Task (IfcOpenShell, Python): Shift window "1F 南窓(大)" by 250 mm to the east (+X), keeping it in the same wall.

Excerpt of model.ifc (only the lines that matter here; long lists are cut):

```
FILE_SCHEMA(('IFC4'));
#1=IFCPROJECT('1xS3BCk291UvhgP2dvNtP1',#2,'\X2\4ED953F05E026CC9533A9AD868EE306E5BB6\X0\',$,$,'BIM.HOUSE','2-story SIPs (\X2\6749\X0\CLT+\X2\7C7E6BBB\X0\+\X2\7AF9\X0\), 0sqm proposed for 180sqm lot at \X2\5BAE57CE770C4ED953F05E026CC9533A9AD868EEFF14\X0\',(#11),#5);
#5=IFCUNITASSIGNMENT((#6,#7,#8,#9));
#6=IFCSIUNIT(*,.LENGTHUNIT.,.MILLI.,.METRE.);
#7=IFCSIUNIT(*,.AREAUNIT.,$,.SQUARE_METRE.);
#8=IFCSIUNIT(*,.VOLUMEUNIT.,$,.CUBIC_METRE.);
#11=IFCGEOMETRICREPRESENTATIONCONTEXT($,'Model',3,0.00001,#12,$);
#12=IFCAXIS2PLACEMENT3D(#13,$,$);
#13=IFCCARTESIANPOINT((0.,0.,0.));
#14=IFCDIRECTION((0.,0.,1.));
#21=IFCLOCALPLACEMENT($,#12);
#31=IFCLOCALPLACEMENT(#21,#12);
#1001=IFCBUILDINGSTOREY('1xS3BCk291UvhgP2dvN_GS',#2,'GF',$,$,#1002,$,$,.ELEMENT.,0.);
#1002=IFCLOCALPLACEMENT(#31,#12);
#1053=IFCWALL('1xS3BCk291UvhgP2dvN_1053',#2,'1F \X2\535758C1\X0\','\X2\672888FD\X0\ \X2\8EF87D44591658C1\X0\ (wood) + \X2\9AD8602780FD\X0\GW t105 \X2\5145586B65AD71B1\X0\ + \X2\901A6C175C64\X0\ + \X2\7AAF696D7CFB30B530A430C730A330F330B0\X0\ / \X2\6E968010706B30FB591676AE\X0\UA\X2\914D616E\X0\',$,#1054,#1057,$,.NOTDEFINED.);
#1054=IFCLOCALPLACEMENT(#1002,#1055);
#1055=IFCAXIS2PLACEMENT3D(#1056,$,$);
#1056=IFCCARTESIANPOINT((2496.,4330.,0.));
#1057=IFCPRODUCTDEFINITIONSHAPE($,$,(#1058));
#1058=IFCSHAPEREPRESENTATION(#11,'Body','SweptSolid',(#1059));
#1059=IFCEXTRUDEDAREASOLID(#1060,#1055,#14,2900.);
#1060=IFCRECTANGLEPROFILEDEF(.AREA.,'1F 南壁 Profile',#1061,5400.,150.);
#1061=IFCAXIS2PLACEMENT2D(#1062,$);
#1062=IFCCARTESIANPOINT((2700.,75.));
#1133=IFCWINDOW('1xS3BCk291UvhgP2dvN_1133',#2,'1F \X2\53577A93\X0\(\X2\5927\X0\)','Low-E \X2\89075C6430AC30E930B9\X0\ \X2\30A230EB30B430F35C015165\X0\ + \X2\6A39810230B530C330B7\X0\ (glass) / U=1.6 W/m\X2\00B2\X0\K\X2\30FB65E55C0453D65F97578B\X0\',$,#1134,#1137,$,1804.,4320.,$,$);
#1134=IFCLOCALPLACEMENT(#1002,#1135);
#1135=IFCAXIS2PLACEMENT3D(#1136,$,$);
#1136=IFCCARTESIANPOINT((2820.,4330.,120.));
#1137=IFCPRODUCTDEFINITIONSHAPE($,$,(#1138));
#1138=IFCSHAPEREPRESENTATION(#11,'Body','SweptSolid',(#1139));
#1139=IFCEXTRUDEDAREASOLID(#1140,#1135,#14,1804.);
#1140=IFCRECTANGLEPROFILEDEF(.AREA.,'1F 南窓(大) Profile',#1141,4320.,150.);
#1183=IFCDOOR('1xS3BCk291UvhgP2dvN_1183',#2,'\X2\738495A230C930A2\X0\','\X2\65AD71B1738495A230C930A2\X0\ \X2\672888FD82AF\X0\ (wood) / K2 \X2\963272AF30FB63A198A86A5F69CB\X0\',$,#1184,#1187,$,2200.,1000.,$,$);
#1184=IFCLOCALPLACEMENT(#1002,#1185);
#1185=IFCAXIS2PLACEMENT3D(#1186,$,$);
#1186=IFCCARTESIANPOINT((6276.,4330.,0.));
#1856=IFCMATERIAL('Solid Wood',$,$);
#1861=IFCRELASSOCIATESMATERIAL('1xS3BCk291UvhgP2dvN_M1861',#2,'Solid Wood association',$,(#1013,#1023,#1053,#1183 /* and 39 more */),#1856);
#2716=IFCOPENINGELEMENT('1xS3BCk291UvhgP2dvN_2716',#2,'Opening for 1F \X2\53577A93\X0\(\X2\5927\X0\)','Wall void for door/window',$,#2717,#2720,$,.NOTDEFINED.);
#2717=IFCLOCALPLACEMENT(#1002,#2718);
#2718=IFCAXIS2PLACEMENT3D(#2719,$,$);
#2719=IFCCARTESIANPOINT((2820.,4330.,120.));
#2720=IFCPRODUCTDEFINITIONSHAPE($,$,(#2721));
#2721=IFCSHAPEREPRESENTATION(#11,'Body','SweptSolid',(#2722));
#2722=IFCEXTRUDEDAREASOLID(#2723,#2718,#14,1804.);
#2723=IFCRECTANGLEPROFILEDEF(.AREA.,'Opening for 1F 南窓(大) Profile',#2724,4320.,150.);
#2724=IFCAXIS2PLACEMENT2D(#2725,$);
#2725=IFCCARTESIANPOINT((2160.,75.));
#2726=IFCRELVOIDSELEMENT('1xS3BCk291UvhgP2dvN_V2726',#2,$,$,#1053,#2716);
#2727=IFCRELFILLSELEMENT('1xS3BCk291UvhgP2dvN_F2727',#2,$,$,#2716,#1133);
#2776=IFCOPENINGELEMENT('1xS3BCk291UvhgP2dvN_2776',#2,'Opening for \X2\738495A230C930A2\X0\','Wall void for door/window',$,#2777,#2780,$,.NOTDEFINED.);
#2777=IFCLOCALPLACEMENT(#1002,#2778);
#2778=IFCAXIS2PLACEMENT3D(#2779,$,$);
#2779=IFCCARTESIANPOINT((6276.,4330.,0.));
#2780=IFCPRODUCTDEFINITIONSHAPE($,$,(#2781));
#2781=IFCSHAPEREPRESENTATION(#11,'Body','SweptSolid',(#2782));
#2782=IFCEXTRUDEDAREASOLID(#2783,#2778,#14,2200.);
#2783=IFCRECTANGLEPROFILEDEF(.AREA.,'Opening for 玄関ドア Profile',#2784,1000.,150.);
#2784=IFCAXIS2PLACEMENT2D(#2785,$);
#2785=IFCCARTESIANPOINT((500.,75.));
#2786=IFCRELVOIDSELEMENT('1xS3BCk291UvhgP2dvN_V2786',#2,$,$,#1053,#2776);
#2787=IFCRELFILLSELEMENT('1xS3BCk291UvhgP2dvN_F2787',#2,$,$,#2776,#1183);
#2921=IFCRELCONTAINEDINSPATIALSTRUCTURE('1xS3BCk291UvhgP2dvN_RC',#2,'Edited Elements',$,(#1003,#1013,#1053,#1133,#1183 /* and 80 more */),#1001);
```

```python
import ifcopenshell
import ifcopenshell.api.geometry
import ifcopenshell.util.placement
import ifcopenshell.util.unit

model = ifcopenshell.open("model.ifc")
unit_scale = ifcopenshell.util.unit.calculate_unit_scale(model)

window = model.by_guid("1xS3BCk291UvhgP2dvN_1133")
opening = window.FillsVoids[0].RelatingOpeningElement
wall = opening.VoidsElements[0].RelatingBuildingElement

wall_matrix = ifcopenshell.util.placement.get_local_placement(wall.ObjectPlacement)
shift = wall_matrix[:3, 0] * 0.25 / unit_scale
before = ifcopenshell.util.placement.get_local_placement(window.ObjectPlacement)[:3, 3].copy()

# The window is not placed relative to its opening, so move both.
for product in (opening, window):
    matrix = ifcopenshell.util.placement.get_local_placement(product.ObjectPlacement)
    matrix[:3, 3] += shift
    ifcopenshell.api.geometry.edit_object_placement(model, product=product, matrix=matrix, is_si=False)

after = ifcopenshell.util.placement.get_local_placement(window.ObjectPlacement)[:3, 3]
print("window moved by", (after - before).round(3) + 0.0)

model.write("model_edited.ifc")
```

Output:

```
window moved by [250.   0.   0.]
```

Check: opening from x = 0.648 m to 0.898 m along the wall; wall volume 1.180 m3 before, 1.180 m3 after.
